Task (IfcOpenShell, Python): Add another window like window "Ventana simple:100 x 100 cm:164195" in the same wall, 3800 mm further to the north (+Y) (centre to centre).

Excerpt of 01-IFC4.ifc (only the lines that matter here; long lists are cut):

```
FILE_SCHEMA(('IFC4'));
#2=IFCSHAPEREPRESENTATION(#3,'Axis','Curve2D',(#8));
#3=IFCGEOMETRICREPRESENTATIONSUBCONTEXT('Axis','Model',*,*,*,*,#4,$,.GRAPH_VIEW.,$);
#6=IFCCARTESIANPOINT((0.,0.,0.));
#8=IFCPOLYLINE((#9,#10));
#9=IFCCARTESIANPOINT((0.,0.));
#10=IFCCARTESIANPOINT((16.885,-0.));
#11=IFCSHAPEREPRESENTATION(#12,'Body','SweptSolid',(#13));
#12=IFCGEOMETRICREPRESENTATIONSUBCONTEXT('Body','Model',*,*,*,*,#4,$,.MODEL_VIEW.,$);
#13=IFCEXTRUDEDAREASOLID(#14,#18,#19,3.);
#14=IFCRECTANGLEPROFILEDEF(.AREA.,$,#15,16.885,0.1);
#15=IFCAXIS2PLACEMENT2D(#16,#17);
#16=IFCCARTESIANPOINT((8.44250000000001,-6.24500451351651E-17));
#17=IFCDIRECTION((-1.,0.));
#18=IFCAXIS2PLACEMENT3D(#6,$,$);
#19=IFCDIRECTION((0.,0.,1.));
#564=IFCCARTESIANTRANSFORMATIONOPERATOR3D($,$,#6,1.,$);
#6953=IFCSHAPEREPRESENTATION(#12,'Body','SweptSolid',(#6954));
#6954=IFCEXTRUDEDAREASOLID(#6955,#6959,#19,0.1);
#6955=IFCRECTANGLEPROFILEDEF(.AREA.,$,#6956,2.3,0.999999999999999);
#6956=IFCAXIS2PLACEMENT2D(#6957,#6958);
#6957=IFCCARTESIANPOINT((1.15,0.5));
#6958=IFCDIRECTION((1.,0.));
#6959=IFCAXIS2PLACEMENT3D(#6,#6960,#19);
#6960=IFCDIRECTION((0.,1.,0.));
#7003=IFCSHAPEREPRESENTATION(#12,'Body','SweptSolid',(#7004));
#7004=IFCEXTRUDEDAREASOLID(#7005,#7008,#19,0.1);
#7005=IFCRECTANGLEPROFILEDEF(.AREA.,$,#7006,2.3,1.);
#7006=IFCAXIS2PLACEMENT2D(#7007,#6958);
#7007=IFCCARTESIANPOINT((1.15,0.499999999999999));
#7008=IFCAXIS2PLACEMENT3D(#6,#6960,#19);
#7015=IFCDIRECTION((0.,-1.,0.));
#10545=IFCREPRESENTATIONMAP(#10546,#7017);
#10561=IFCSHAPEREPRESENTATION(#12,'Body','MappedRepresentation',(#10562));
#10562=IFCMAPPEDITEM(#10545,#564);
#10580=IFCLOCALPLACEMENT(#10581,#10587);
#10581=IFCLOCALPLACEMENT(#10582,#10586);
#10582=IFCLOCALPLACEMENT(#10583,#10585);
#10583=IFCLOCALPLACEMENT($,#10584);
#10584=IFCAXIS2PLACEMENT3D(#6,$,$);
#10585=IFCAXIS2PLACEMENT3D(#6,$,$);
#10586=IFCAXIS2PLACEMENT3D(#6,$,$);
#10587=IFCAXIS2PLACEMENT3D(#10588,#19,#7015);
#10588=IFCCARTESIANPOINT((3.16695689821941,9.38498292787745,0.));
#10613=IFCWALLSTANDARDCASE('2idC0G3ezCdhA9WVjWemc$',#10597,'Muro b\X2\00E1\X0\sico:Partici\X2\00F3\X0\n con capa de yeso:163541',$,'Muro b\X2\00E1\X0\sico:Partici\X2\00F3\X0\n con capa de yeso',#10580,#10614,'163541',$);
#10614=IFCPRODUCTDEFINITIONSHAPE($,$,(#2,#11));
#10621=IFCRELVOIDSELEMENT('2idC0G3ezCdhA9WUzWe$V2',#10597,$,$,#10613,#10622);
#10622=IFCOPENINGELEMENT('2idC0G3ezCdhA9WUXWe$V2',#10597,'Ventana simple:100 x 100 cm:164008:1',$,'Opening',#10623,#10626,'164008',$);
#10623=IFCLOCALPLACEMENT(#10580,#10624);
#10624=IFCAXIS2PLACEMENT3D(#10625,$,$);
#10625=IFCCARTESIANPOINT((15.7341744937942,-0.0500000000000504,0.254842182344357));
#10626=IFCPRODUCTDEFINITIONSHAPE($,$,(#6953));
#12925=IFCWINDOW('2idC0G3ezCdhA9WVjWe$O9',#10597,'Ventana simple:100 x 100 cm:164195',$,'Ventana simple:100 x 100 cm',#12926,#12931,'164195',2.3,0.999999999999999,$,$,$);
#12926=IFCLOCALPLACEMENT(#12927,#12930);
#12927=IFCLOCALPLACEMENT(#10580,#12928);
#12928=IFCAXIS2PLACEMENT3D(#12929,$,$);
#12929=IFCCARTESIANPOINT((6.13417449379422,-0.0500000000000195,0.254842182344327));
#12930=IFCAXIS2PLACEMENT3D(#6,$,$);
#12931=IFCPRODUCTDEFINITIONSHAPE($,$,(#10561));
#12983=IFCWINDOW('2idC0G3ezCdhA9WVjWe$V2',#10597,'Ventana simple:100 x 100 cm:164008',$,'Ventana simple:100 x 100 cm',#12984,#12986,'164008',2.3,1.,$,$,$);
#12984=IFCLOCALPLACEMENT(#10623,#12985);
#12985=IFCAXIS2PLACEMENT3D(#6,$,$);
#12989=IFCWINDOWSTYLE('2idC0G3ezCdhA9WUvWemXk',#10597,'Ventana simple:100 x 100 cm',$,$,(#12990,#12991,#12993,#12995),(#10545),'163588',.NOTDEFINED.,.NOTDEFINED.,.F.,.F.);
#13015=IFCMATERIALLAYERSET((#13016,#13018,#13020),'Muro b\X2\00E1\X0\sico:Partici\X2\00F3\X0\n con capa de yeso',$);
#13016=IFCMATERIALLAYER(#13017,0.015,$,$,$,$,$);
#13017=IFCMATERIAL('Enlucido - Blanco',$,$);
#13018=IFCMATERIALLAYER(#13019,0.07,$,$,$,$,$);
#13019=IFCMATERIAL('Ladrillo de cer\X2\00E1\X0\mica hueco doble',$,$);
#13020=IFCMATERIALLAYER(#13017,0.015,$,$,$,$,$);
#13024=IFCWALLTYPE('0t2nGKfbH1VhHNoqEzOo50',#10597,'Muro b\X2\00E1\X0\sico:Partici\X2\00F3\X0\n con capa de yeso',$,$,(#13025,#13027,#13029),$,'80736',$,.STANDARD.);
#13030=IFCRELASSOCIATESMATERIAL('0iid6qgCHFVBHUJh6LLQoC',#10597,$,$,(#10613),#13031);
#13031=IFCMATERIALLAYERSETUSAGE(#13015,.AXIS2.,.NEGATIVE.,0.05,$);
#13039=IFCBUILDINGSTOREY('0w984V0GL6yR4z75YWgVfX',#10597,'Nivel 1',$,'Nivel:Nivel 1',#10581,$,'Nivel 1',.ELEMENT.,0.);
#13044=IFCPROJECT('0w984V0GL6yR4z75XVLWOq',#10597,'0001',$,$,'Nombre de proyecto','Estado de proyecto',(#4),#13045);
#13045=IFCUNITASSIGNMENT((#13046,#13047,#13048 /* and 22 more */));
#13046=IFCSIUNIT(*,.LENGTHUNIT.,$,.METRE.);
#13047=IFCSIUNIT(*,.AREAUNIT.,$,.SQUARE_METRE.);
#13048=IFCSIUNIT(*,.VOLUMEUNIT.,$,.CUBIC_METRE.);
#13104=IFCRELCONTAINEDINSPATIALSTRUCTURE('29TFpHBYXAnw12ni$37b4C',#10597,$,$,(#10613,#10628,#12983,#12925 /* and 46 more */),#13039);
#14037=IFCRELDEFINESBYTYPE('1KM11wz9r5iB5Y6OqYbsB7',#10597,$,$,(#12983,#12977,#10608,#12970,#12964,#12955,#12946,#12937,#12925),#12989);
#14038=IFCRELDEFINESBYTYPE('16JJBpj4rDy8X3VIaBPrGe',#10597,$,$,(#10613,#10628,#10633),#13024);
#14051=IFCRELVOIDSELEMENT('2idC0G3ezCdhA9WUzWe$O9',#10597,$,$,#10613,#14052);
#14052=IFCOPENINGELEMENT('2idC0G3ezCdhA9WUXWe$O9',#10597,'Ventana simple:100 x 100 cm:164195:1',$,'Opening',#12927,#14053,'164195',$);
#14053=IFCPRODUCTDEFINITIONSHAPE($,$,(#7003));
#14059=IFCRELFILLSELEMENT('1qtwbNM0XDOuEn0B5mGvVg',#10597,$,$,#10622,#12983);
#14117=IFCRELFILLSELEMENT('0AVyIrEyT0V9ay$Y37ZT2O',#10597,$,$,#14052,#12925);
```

```python
import ifcopenshell
import ifcopenshell.api.feature
import ifcopenshell.api.geometry
import ifcopenshell.api.root
import ifcopenshell.geom
import ifcopenshell.util.element
import ifcopenshell.util.placement
import ifcopenshell.util.shape
import ifcopenshell.util.unit

model = ifcopenshell.open("01-IFC4.ifc")
unit_scale = ifcopenshell.util.unit.calculate_unit_scale(model)
settings = ifcopenshell.geom.settings()


def volume(element):
    """Net volume in cubic metres, openings subtracted."""
    shape = ifcopenshell.geom.create_shape(settings, element)
    return ifcopenshell.util.shape.get_volume(shape.geometry)


def reuse_history(source, copy):
    """copy_class also copies each property set's owner history, people and application; keep the originals."""
    for rel in copy.IsDefinedBy:
        if rel.is_a("IfcRelDefinesByProperties") and (history := rel.RelatingPropertyDefinition.OwnerHistory):
            rel.RelatingPropertyDefinition.OwnerHistory = source.OwnerHistory
            ifcopenshell.util.element.remove_deep2(model, history)


window = model.by_id(12925)
opening = window.FillsVoids[0].RelatingOpeningElement
wall = opening.VoidsElements[0].RelatingBuildingElement
before = volume(wall)
shift = ifcopenshell.util.placement.get_local_placement(wall.ObjectPlacement)[:3, 0] * -3.8 / unit_scale

# copy_class copies the void relationship, type, container and properties, but no geometry.
new_opening = ifcopenshell.api.root.copy_class(model, product=opening)
new_opening.Representation = ifcopenshell.util.element.copy_deep(
    model, opening.Representation, exclude=["IfcGeometricRepresentationContext", "IfcRepresentationMap"]
)
new_opening.Name = "Ventana simple:100 x 100 cm"
new_opening.Tag = None
new_window = ifcopenshell.api.root.copy_class(model, product=window)
new_window.Representation = ifcopenshell.util.element.copy_deep(
    model, window.Representation, exclude=["IfcGeometricRepresentationContext", "IfcRepresentationMap"]
)
new_window.Name = "Ventana simple:100 x 100 cm"
new_window.Tag = None
reuse_history(window, new_window)
ifcopenshell.api.feature.add_filling(model, opening=new_opening, element=new_window)

for old, new in ((opening, new_opening), (window, new_window)):
    matrix = ifcopenshell.util.placement.get_local_placement(old.ObjectPlacement)
    matrix[:3, 3] += shift
    ifcopenshell.api.geometry.edit_object_placement(model, product=new, matrix=matrix, is_si=False)

after = volume(wall)

print(f"wall volume {before:.3f} -> {after:.3f} m3")

model.write("01-IFC4_rev.ifc")
```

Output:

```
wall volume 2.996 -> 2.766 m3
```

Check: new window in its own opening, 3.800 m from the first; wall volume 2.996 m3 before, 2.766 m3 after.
